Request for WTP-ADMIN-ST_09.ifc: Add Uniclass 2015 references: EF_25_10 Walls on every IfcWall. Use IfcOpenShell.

First a look at what the model holds.

```python
import ifcopenshell

model = ifcopenshell.open("WTP-ADMIN-ST_09.ifc")
print(model.schema)
print("classifications:", [c.Name for c in model.by_type("IfcClassification")])
for ifc_class in ("IfcDoor", "IfcRoof", "IfcStair", "IfcWall", "IfcWindow"):
    print(ifc_class, len(model.by_type(ifc_class)))
```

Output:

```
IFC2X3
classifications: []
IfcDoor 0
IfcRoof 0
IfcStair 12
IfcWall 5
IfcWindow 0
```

```python
import ifcopenshell
import ifcopenshell.api.classification

model = ifcopenshell.open("WTP-ADMIN-ST_09.ifc")

# IFC2X3 requires Source and Edition and has no link from the project to the system.
system = model.create_entity("IfcClassification", Source="NBS", Edition="2015", Name="Uniclass 2015")

codes = {
    "IfcWall": ("EF_25_10", "Walls"),
}
for ifc_class, (code, name) in codes.items():
    products = model.by_type(ifc_class)
    ifcopenshell.api.classification.add_reference(
        model, products=products, classification=system, identification=code, name=name
    )
    print(code, len(products))

model.write("WTP-ADMIN-ST_09_rev.ifc")
```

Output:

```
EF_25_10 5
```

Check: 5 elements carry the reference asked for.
